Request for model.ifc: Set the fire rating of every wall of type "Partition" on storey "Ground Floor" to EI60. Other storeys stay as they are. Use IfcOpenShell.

First a look at what the model holds.

```python
import ifcopenshell
import ifcopenshell.util.element

model = ifcopenshell.open("model.ifc")
print(model.schema)
storey = next(s for s in model.by_type("IfcBuildingStorey") if s.Name == "Ground Floor")
walls = [e for e in ifcopenshell.util.element.get_decomposition(storey) if e.is_a("IfcWall")]
seen = {}
for e in walls:
    element_type = ifcopenshell.util.element.get_type(e)
    key = (element_type.Name if element_type != e and element_type else None, ifcopenshell.util.element.get_pset(e, "Pset_WallCommon", "FireRating"))
    seen[key] = seen.get(key, 0) + 1
for (name, value), count in sorted(seen.items(), key=str):
    print(count, "x", name, "|", value)
```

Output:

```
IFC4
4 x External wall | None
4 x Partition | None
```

```python
import ifcopenshell
import ifcopenshell.api.pset
import ifcopenshell.util.element

model = ifcopenshell.open("model.ifc")

storey = next(s for s in model.by_type("IfcBuildingStorey") if s.Name == "Ground Floor")
walls = [e for e in ifcopenshell.util.element.get_decomposition(storey) if e.is_a("IfcWall")]

count = 0
for e in walls:
    element_type = ifcopenshell.util.element.get_type(e)
    if element_type in (None, e) or element_type.Name != "Partition":
        continue
    # add_pset returns the element's existing set when there is one.
    pset = ifcopenshell.api.pset.add_pset(model, product=e, name="Pset_WallCommon")
    ifcopenshell.api.pset.edit_pset(model, pset=pset, properties={"FireRating": "EI60"})
    count += 1

print(count, "walls updated")

model.write("model-out.ifc")
```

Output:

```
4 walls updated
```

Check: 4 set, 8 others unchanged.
